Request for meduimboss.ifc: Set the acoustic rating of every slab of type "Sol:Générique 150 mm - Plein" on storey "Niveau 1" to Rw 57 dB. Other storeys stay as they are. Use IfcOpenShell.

First a look at what the model holds.

```python
import ifcopenshell
import ifcopenshell.util.element

model = ifcopenshell.open("meduimboss.ifc")
print(model.schema)
storey = next(s for s in model.by_type("IfcBuildingStorey") if s.Name == "Niveau 1")
slabs = [e for e in ifcopenshell.util.element.get_decomposition(storey) if e.is_a("IfcSlab")]
seen = {}
for e in slabs:
    element_type = ifcopenshell.util.element.get_type(e)
    key = (element_type.Name if element_type != e and element_type else None, ifcopenshell.util.element.get_pset(e, "Pset_SlabCommon", "AcousticRating"))
    seen[key] = seen.get(key, 0) + 1
for (name, value), count in sorted(seen.items(), key=str):
    print(count, "x", name, "|", value)
```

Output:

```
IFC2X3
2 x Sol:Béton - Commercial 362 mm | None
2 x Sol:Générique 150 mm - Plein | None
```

```python
import ifcopenshell
import ifcopenshell.api.pset
import ifcopenshell.util.element

model = ifcopenshell.open("meduimboss.ifc")

storey = next(s for s in model.by_type("IfcBuildingStorey") if s.Name == "Niveau 1")
slabs = [e for e in ifcopenshell.util.element.get_decomposition(storey) if e.is_a("IfcSlab")]

count = 0
for e in slabs:
    element_type = ifcopenshell.util.element.get_type(e)
    if element_type in (None, e) or element_type.Name != "Sol:Générique 150 mm - Plein":
        continue
    # add_pset returns the element's existing set when there is one.
    pset = ifcopenshell.api.pset.add_pset(model, product=e, name="Pset_SlabCommon")
    ifcopenshell.api.pset.edit_pset(model, pset=pset, properties={"AcousticRating": "Rw 57 dB"})
    count += 1

print(count, "slabs updated")

model.write("meduimboss_rev.ifc")
```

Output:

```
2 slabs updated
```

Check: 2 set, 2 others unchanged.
